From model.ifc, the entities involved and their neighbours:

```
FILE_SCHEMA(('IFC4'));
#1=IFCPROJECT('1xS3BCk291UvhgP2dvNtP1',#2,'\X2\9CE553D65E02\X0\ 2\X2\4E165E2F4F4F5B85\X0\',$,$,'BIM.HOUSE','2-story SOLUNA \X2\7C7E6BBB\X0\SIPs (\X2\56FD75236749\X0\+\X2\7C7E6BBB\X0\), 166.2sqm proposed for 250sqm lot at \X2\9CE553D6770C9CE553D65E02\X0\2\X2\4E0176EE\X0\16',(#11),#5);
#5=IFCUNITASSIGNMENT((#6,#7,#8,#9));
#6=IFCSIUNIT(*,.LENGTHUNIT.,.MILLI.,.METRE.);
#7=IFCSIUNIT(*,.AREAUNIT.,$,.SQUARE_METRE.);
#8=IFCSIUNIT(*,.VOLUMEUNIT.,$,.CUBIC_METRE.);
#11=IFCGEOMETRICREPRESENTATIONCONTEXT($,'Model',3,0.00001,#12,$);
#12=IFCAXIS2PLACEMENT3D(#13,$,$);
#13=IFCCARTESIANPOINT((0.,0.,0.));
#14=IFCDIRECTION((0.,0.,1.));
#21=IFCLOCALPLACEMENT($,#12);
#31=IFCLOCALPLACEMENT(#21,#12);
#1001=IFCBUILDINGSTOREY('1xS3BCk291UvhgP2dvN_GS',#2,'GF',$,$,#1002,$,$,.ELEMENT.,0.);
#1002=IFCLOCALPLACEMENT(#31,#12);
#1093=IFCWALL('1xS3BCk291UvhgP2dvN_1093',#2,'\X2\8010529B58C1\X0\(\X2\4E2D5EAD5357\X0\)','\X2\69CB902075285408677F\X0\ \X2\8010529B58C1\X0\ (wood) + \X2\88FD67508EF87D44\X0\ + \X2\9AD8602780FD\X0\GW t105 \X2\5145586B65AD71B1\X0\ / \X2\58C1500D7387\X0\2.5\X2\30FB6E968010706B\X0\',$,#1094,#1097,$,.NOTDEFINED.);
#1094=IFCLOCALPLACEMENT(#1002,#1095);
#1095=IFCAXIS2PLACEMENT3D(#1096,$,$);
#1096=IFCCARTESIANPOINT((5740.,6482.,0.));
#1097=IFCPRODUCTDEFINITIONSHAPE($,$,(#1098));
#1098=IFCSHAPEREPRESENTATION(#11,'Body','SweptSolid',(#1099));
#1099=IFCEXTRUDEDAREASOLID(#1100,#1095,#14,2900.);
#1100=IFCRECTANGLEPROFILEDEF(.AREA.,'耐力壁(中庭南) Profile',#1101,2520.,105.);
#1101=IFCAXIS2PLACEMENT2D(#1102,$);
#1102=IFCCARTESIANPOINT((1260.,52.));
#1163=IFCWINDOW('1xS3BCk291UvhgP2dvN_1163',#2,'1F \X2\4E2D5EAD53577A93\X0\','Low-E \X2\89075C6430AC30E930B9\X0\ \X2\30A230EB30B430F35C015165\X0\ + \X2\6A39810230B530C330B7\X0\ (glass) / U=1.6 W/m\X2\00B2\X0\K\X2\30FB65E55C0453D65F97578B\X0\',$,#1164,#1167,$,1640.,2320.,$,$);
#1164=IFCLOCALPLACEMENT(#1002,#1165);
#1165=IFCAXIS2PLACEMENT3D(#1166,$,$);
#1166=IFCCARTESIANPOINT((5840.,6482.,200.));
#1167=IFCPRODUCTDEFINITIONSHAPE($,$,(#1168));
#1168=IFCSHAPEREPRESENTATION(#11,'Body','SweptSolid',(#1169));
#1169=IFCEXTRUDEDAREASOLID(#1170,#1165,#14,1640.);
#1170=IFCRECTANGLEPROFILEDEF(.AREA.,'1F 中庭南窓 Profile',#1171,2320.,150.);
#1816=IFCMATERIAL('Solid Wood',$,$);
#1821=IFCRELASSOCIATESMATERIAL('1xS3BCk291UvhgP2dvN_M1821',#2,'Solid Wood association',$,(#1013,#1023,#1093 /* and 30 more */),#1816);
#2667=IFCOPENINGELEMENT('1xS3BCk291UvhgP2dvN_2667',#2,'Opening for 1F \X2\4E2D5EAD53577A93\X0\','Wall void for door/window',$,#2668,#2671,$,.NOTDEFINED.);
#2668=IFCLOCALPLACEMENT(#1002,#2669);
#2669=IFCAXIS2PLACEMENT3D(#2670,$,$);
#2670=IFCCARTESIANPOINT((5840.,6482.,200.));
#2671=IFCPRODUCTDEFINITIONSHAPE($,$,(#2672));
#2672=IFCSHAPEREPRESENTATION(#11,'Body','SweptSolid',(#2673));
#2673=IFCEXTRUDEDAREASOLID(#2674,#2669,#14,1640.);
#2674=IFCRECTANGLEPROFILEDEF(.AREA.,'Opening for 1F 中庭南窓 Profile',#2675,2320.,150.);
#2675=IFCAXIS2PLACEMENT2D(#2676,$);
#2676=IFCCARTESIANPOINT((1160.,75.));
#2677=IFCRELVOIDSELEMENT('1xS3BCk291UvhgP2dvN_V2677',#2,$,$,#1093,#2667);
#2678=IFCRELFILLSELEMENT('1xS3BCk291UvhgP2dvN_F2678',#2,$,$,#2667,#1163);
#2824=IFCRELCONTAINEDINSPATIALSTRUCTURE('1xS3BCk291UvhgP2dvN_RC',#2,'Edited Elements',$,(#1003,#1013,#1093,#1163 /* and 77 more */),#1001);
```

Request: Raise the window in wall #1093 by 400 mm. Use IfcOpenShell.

```python
import numpy as np
import ifcopenshell
import ifcopenshell.api.geometry
import ifcopenshell.util.placement
import ifcopenshell.util.unit

model = ifcopenshell.open("model.ifc")
unit_scale = ifcopenshell.util.unit.calculate_unit_scale(model)

window = model.by_guid("1xS3BCk291UvhgP2dvN_1163")
opening = window.FillsVoids[0].RelatingOpeningElement
dz = 400.0

shift = np.array([0.0, 0.0, dz])
# The window is not placed relative to its opening, so move both.
for product in (opening, window):
    matrix = ifcopenshell.util.placement.get_local_placement(product.ObjectPlacement)
    matrix[:3, 3] += shift
    ifcopenshell.api.geometry.edit_object_placement(model, product=product, matrix=matrix, is_si=False)

print(f"moved by {dz * unit_scale:+.3f} m")

model.write("model_rev.ifc")
```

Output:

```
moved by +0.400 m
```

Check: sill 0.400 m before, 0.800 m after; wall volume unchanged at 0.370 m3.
